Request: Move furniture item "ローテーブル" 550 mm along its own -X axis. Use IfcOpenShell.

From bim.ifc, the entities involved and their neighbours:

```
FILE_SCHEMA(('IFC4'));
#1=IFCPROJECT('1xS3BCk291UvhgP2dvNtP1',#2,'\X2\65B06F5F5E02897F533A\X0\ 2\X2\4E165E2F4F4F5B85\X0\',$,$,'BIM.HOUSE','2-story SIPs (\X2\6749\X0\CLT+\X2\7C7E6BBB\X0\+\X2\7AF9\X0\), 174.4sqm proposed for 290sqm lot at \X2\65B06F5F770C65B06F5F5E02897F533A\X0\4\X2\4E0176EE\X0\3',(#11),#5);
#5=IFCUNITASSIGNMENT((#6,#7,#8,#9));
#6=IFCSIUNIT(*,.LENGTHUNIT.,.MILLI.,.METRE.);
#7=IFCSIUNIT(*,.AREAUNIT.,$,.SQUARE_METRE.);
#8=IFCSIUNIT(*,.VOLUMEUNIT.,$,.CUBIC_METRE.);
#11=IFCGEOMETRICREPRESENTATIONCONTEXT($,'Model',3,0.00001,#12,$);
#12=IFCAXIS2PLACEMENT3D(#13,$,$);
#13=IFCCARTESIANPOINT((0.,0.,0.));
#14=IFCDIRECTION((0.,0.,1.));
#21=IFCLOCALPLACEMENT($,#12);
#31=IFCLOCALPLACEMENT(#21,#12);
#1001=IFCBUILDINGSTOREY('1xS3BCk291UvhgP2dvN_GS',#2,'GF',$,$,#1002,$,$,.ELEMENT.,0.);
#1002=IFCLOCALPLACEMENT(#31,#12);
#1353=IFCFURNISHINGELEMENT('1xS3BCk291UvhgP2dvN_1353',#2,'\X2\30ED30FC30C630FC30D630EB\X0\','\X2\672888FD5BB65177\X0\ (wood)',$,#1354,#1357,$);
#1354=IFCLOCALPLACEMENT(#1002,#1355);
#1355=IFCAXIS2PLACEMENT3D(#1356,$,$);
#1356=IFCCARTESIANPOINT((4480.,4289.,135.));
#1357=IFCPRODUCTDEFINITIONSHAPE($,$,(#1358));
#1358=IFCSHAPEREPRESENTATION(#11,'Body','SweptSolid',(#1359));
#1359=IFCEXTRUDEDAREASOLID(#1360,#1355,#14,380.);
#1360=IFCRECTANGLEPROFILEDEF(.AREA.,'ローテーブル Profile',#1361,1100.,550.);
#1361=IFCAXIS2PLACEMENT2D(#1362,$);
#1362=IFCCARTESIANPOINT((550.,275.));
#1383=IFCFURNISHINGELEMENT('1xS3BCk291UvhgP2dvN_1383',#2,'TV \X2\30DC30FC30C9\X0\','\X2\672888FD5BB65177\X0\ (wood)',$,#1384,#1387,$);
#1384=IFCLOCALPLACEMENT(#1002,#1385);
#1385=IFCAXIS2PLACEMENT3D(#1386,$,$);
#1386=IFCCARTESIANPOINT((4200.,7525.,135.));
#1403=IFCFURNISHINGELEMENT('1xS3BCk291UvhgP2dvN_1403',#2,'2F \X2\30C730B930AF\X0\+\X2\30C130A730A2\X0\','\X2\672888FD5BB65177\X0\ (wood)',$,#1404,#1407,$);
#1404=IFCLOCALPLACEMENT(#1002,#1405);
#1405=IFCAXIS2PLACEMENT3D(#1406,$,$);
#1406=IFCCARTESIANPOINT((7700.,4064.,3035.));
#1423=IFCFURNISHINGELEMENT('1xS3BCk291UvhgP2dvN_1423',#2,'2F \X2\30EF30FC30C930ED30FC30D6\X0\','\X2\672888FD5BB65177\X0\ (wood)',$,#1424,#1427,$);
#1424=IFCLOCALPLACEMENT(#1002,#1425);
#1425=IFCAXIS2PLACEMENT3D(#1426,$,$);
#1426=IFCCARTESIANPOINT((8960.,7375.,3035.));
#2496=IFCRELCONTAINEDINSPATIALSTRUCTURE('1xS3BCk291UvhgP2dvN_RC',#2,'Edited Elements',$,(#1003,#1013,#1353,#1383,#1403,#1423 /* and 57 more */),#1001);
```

```python
import ifcopenshell
import ifcopenshell.api.geometry
import ifcopenshell.util.placement
import ifcopenshell.util.unit

model = ifcopenshell.open("bim.ifc")
unit_scale = ifcopenshell.util.unit.calculate_unit_scale(model)

item = model.by_id(1353)
matrix = ifcopenshell.util.placement.get_local_placement(item.ObjectPlacement)
matrix[:3, 3] -= matrix[:3, 0] * 0.55 / unit_scale
ifcopenshell.api.geometry.edit_object_placement(model, product=item, matrix=matrix, is_si=False)

print(ifcopenshell.util.placement.get_local_placement(item.ObjectPlacement).round(3) + 0.0)

model.write("bim_updated.ifc")
```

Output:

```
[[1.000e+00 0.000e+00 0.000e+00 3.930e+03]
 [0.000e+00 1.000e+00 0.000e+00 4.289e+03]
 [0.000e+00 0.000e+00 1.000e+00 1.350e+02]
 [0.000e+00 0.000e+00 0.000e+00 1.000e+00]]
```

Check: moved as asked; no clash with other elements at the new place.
